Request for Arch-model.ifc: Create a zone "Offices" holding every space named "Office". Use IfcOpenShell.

First a look at what the model holds.

```python
import ifcopenshell

model = ifcopenshell.open("Arch-model.ifc")
print(model.schema)
seen = {}
for space in model.by_type("IfcSpace"):
    seen[space.LongName] = seen.get(space.LongName, 0) + 1
for name, count in sorted(seen.items(), key=str):
    print(count, "x", name)
print("zones:", [z.Name for z in model.by_type("IfcZone")][:20])
```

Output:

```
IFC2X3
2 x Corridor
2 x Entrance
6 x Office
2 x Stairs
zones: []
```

```python
import ifcopenshell
import ifcopenshell.api.group
import ifcopenshell.api.root

model = ifcopenshell.open("Arch-model.ifc")

names = {"Office"}
spaces = [s for s in model.by_type("IfcSpace") if s.LongName in names]

zone = ifcopenshell.api.root.create_entity(model, ifc_class="IfcZone", name="Offices")
ifcopenshell.api.group.assign_group(model, products=spaces, group=zone)
print(len(spaces), "spaces in", zone.Name)

model.write("Arch-model_updated.ifc")
```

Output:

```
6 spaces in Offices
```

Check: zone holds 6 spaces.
